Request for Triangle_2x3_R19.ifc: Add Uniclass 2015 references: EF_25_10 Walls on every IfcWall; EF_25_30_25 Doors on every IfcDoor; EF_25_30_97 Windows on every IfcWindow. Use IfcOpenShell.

First a look at what the model holds.

```python
import ifcopenshell

model = ifcopenshell.open("Triangle_2x3_R19.ifc")
print(model.schema)
print("classifications:", [c.Name for c in model.by_type("IfcClassification")])
for ifc_class in ("IfcDoor", "IfcRoof", "IfcStair", "IfcWall", "IfcWindow"):
    print(ifc_class, len(model.by_type(ifc_class)))
```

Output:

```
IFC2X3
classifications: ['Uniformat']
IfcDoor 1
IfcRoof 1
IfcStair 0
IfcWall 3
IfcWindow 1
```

```python
import ifcopenshell
import ifcopenshell.api.classification

model = ifcopenshell.open("Triangle_2x3_R19.ifc")

# IFC2X3 requires Source and Edition and has no link from the project to the system.
system = model.create_entity("IfcClassification", Source="NBS", Edition="2015", Name="Uniclass 2015")

codes = {
    "IfcWall": ("EF_25_10", "Walls"),
    "IfcDoor": ("EF_25_30_25", "Doors"),
    "IfcWindow": ("EF_25_30_97", "Windows"),
}
for ifc_class, (code, name) in codes.items():
    products = model.by_type(ifc_class)
    ifcopenshell.api.classification.add_reference(
        model, products=products, classification=system, identification=code, name=name
    )
    print(code, len(products))

model.write("Triangle_2x3_R19_v2.ifc")
```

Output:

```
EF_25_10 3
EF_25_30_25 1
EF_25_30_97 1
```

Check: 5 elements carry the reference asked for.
